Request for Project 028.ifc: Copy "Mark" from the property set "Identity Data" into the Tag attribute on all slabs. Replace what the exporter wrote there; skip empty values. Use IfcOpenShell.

First a look at what the model holds.

```python
import ifcopenshell
import ifcopenshell.util.element

model = ifcopenshell.open("Project 028.ifc")
print(model.schema)
slabs = model.by_type("IfcSlab")
print(len(slabs), "slabs")
for e in slabs[:8]:
    source = ifcopenshell.util.element.get_pset(e, "Identity Data", "Mark")
    target = e.Tag
    print(e.id(), repr(source), repr(target), sep=" | ")
```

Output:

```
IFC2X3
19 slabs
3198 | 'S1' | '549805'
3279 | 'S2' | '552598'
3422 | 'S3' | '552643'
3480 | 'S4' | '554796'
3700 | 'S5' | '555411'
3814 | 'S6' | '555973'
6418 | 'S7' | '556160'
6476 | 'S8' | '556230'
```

```python
import ifcopenshell
import ifcopenshell.util.element

model = ifcopenshell.open("Project 028.ifc")

count = 0
for e in model.by_type("IfcSlab"):
    value = ifcopenshell.util.element.get_pset(e, "Identity Data", "Mark")
    current = e.Tag
    if not value or not value.strip() or current == value:
        continue
    e.Tag = value
    count += 1

print(count, "slabs updated")

model.write("Project 028_edited.ifc")
```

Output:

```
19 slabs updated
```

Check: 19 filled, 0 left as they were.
